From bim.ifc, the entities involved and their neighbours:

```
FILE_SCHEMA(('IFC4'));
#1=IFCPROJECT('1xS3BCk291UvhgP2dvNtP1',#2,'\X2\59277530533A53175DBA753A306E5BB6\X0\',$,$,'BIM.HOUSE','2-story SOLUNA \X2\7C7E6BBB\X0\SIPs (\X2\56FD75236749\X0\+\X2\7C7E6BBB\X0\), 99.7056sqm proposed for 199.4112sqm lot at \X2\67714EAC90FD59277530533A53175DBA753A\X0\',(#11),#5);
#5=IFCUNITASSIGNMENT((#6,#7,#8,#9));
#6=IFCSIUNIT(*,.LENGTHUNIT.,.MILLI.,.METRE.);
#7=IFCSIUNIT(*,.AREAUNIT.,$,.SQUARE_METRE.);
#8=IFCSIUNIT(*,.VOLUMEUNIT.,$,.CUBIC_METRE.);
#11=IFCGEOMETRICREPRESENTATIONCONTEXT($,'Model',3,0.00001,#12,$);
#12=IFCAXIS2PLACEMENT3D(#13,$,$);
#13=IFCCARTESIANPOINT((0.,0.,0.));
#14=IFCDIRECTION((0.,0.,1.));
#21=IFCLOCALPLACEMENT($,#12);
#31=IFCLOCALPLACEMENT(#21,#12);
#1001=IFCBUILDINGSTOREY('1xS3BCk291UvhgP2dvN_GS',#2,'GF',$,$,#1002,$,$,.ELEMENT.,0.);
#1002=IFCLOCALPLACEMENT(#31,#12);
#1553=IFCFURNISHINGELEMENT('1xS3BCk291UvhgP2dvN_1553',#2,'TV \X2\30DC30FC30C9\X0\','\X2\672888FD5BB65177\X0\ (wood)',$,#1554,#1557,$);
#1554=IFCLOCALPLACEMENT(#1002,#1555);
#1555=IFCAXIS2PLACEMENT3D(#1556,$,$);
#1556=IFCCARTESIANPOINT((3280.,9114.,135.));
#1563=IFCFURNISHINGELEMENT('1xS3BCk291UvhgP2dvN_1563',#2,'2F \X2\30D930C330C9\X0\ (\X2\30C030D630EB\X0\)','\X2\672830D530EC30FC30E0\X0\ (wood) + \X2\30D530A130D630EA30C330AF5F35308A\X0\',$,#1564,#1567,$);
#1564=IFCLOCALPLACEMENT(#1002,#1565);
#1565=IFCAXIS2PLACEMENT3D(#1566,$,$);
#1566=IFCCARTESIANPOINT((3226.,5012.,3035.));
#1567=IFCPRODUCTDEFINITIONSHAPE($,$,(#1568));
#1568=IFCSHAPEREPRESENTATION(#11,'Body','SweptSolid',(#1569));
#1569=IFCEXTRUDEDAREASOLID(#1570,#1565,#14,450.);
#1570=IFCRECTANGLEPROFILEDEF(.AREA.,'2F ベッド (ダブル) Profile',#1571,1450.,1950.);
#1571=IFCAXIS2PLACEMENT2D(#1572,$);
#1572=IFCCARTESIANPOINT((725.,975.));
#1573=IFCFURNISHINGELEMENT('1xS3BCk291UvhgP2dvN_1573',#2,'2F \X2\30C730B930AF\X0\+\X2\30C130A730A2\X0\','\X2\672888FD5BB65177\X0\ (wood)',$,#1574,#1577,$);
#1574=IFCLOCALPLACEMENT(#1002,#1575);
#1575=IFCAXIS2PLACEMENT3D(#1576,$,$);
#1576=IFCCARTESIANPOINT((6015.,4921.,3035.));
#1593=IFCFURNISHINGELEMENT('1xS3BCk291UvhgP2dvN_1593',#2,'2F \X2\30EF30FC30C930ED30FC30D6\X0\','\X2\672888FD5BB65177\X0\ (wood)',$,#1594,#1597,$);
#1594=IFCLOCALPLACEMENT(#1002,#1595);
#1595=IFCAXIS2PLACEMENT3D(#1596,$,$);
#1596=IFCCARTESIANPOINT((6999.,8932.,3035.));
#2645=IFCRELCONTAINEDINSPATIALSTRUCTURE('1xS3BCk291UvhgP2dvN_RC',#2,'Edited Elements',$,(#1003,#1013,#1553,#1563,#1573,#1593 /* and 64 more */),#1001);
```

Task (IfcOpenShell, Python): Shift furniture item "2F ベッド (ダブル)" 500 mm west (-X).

```python
import ifcopenshell
import ifcopenshell.api.geometry
import ifcopenshell.util.placement
import ifcopenshell.util.unit

model = ifcopenshell.open("bim.ifc")
unit_scale = ifcopenshell.util.unit.calculate_unit_scale(model)

item = model.by_guid("1xS3BCk291UvhgP2dvN_1563")
matrix = ifcopenshell.util.placement.get_local_placement(item.ObjectPlacement)
matrix[0, 3] -= 0.5 / unit_scale
ifcopenshell.api.geometry.edit_object_placement(model, product=item, matrix=matrix, is_si=False)

print(ifcopenshell.util.placement.get_local_placement(item.ObjectPlacement).round(3) + 0.0)

model.write("bim_v2.ifc")
```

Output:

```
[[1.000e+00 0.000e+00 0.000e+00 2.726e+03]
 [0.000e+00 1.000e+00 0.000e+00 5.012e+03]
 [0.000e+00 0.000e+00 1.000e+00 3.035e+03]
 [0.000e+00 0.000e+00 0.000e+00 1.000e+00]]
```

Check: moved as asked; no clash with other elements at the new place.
